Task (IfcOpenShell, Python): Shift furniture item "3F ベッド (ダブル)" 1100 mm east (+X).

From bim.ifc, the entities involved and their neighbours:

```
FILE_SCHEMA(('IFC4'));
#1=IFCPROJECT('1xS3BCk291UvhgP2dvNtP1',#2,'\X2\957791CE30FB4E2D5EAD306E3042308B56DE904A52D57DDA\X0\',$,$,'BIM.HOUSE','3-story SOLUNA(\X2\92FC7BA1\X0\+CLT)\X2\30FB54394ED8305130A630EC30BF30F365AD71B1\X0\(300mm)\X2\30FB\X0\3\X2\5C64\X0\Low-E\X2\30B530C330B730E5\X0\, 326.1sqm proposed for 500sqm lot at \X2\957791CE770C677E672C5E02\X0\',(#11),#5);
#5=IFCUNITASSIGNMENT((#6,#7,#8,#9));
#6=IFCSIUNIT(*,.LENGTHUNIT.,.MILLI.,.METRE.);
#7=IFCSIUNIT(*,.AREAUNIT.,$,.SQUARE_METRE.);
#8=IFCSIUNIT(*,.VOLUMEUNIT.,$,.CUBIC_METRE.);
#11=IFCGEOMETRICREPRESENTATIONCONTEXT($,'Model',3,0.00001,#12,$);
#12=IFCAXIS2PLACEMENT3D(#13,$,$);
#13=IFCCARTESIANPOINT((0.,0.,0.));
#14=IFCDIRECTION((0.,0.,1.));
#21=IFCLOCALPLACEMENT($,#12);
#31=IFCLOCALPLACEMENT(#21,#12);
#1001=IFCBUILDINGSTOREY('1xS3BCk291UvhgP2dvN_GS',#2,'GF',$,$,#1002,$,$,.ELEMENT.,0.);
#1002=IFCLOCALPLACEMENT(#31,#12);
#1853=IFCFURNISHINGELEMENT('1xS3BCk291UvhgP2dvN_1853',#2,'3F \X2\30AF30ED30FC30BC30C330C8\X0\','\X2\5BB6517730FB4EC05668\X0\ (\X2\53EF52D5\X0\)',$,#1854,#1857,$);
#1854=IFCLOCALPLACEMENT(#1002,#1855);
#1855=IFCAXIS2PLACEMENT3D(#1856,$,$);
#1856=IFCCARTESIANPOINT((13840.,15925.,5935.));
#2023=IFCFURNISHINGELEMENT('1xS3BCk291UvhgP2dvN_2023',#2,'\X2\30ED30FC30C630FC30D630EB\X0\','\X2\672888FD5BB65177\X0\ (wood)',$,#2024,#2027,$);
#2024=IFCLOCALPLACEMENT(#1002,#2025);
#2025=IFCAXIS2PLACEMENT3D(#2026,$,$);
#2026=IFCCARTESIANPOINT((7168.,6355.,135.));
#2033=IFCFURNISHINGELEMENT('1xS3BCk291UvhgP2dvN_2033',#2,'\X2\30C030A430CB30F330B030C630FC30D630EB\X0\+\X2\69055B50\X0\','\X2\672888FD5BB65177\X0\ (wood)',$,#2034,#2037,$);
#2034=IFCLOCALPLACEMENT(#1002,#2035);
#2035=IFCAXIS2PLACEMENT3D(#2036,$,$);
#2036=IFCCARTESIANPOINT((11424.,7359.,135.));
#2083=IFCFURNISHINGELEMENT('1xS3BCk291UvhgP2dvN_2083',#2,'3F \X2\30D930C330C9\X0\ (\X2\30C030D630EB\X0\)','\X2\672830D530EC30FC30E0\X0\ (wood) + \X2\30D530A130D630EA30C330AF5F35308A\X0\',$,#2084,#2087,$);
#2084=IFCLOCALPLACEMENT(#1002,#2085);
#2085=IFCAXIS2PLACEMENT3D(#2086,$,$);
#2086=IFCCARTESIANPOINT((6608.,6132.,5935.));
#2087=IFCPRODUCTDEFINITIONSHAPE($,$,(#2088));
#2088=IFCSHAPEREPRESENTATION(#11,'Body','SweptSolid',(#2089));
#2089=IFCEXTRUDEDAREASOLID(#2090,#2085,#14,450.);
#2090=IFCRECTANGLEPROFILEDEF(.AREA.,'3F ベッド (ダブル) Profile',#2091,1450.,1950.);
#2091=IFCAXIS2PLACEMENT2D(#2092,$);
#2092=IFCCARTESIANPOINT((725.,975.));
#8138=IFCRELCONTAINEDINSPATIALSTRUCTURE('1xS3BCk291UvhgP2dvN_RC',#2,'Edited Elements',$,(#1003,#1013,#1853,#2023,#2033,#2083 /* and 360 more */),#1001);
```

```python
import ifcopenshell
import ifcopenshell.api.geometry
import ifcopenshell.util.placement
import ifcopenshell.util.unit

model = ifcopenshell.open("bim.ifc")
unit_scale = ifcopenshell.util.unit.calculate_unit_scale(model)

item = model.by_guid("1xS3BCk291UvhgP2dvN_2083")
matrix = ifcopenshell.util.placement.get_local_placement(item.ObjectPlacement)
matrix[0, 3] += 1.1 / unit_scale
ifcopenshell.api.geometry.edit_object_placement(model, product=item, matrix=matrix, is_si=False)

print(ifcopenshell.util.placement.get_local_placement(item.ObjectPlacement).round(3) + 0.0)

model.write("bim-out.ifc")
```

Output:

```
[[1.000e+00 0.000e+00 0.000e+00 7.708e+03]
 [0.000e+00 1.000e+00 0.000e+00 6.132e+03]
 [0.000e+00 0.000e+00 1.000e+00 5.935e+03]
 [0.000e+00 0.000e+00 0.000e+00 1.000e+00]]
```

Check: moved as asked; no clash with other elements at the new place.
